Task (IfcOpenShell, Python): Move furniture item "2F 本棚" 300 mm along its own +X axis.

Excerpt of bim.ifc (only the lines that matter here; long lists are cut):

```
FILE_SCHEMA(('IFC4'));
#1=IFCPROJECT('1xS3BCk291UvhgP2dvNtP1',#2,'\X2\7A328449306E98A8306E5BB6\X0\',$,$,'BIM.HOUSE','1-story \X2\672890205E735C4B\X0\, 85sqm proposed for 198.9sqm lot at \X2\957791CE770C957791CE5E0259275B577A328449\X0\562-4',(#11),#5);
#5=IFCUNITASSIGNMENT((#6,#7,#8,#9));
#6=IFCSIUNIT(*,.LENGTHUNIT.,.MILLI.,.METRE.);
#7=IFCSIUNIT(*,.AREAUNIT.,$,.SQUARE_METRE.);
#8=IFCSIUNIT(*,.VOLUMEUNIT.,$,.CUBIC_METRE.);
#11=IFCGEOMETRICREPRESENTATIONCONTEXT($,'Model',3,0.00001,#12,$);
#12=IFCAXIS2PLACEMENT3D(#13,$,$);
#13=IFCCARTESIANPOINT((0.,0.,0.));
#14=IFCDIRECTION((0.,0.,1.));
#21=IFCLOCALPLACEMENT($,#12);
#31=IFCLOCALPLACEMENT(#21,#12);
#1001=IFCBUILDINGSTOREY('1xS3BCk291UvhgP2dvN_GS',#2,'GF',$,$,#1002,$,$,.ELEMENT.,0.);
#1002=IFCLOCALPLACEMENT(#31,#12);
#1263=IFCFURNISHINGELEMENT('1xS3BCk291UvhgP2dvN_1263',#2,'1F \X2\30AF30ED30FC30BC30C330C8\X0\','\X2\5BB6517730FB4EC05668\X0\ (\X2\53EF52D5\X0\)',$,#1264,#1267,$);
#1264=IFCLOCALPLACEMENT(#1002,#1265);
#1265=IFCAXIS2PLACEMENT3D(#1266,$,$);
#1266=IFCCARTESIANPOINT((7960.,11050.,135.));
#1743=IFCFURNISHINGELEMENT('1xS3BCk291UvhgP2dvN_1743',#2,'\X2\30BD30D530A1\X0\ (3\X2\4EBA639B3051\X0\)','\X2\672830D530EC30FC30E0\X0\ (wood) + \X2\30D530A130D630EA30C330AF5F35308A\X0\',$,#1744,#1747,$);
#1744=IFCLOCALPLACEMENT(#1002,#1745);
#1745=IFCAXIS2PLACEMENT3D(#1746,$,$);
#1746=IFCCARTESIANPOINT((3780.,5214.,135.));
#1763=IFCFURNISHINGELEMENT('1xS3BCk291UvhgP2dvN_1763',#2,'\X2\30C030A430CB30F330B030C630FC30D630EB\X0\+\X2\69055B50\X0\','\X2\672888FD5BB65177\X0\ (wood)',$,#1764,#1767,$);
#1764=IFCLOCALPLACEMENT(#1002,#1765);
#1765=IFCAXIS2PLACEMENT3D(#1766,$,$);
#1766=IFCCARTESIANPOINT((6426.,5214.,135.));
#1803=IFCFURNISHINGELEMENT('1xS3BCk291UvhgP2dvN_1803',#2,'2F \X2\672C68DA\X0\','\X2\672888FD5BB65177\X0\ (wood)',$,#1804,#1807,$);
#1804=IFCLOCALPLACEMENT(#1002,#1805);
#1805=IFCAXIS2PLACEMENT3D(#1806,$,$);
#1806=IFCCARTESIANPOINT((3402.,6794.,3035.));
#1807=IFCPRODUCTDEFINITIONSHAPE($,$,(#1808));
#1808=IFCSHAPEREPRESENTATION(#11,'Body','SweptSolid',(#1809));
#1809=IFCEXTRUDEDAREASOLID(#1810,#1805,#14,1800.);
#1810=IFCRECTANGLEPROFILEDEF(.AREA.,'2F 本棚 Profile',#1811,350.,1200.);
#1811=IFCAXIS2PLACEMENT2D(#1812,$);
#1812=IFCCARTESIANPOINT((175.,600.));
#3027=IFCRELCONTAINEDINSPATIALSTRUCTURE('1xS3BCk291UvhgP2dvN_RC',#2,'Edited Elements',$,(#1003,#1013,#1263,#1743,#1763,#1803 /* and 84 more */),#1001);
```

```python
import ifcopenshell
import ifcopenshell.api.geometry
import ifcopenshell.util.placement

model = ifcopenshell.open("bim.ifc")

item = model.by_id(1803)
matrix = ifcopenshell.util.placement.get_local_placement(item.ObjectPlacement)
matrix[:3, 3] += matrix[:3, 0] * 300.0
ifcopenshell.api.geometry.edit_object_placement(model, product=item, matrix=matrix, is_si=False)

print(ifcopenshell.util.placement.get_local_placement(item.ObjectPlacement).round(3) + 0.0)

model.write("bim_updated.ifc")
```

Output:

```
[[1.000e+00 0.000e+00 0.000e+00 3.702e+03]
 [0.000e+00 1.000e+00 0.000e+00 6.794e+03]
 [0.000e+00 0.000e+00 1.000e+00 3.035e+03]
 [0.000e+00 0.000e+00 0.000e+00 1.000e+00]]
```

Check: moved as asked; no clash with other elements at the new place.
